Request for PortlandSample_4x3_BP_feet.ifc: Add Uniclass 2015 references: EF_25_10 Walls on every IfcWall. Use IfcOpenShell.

First a look at what the model holds.

```python
import ifcopenshell

model = ifcopenshell.open("PortlandSample_4x3_BP_feet.ifc")
print(model.schema)
print("classifications:", [c.Name for c in model.by_type("IfcClassification")])
for ifc_class in ("IfcDoor", "IfcRoof", "IfcStair", "IfcWall", "IfcWindow"):
    print(ifc_class, len(model.by_type(ifc_class)))
```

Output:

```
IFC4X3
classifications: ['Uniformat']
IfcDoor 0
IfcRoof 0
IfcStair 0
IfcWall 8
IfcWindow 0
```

```python
import ifcopenshell
import ifcopenshell.api.classification

model = ifcopenshell.open("PortlandSample_4x3_BP_feet.ifc")

system = ifcopenshell.api.classification.add_classification(model, classification="Uniclass 2015")

codes = {
    "IfcWall": ("EF_25_10", "Walls"),
}
for ifc_class, (code, name) in codes.items():
    products = model.by_type(ifc_class)
    ifcopenshell.api.classification.add_reference(
        model, products=products, classification=system, identification=code, name=name
    )
    print(code, len(products))

model.write("PortlandSample_4x3_BP_feet-out.ifc")
```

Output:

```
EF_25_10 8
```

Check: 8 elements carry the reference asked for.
